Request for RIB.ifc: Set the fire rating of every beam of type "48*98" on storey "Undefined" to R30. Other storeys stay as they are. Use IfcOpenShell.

First a look at what the model holds.

```python
import ifcopenshell
import ifcopenshell.util.element

model = ifcopenshell.open("RIB.ifc")
print(model.schema)
storey = next(s for s in model.by_type("IfcBuildingStorey") if s.Name == "Undefined")
beams = [e for e in ifcopenshell.util.element.get_decomposition(storey) if e.is_a("IfcBeam")]
seen = {}
for e in beams:
    element_type = ifcopenshell.util.element.get_type(e)
    key = (element_type.Name if element_type != e and element_type else None, ifcopenshell.util.element.get_pset(e, "Pset_BeamCommon", "FireRating"))
    seen[key] = seen.get(key, 0) + 1
for (name, value), count in sorted(seen.items(), key=str):
    print(count, "x", name, "|", value)
```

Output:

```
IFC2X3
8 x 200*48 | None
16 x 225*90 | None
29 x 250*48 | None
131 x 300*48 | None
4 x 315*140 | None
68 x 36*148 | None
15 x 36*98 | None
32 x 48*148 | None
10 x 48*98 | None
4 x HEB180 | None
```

```python
import ifcopenshell
import ifcopenshell.api.pset
import ifcopenshell.util.element

model = ifcopenshell.open("RIB.ifc")

storey = next(s for s in model.by_type("IfcBuildingStorey") if s.Name == "Undefined")
beams = [e for e in ifcopenshell.util.element.get_decomposition(storey) if e.is_a("IfcBeam")]

count = 0
for e in beams:
    element_type = ifcopenshell.util.element.get_type(e)
    if element_type in (None, e) or element_type.Name != "48*98":
        continue
    # add_pset returns the element's existing set when there is one.
    pset = ifcopenshell.api.pset.add_pset(model, product=e, name="Pset_BeamCommon")
    ifcopenshell.api.pset.edit_pset(model, pset=pset, properties={"FireRating": "R30"})
    count += 1

print(count, "beams updated")

model.write("RIB_updated.ifc")
```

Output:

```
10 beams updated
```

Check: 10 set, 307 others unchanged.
